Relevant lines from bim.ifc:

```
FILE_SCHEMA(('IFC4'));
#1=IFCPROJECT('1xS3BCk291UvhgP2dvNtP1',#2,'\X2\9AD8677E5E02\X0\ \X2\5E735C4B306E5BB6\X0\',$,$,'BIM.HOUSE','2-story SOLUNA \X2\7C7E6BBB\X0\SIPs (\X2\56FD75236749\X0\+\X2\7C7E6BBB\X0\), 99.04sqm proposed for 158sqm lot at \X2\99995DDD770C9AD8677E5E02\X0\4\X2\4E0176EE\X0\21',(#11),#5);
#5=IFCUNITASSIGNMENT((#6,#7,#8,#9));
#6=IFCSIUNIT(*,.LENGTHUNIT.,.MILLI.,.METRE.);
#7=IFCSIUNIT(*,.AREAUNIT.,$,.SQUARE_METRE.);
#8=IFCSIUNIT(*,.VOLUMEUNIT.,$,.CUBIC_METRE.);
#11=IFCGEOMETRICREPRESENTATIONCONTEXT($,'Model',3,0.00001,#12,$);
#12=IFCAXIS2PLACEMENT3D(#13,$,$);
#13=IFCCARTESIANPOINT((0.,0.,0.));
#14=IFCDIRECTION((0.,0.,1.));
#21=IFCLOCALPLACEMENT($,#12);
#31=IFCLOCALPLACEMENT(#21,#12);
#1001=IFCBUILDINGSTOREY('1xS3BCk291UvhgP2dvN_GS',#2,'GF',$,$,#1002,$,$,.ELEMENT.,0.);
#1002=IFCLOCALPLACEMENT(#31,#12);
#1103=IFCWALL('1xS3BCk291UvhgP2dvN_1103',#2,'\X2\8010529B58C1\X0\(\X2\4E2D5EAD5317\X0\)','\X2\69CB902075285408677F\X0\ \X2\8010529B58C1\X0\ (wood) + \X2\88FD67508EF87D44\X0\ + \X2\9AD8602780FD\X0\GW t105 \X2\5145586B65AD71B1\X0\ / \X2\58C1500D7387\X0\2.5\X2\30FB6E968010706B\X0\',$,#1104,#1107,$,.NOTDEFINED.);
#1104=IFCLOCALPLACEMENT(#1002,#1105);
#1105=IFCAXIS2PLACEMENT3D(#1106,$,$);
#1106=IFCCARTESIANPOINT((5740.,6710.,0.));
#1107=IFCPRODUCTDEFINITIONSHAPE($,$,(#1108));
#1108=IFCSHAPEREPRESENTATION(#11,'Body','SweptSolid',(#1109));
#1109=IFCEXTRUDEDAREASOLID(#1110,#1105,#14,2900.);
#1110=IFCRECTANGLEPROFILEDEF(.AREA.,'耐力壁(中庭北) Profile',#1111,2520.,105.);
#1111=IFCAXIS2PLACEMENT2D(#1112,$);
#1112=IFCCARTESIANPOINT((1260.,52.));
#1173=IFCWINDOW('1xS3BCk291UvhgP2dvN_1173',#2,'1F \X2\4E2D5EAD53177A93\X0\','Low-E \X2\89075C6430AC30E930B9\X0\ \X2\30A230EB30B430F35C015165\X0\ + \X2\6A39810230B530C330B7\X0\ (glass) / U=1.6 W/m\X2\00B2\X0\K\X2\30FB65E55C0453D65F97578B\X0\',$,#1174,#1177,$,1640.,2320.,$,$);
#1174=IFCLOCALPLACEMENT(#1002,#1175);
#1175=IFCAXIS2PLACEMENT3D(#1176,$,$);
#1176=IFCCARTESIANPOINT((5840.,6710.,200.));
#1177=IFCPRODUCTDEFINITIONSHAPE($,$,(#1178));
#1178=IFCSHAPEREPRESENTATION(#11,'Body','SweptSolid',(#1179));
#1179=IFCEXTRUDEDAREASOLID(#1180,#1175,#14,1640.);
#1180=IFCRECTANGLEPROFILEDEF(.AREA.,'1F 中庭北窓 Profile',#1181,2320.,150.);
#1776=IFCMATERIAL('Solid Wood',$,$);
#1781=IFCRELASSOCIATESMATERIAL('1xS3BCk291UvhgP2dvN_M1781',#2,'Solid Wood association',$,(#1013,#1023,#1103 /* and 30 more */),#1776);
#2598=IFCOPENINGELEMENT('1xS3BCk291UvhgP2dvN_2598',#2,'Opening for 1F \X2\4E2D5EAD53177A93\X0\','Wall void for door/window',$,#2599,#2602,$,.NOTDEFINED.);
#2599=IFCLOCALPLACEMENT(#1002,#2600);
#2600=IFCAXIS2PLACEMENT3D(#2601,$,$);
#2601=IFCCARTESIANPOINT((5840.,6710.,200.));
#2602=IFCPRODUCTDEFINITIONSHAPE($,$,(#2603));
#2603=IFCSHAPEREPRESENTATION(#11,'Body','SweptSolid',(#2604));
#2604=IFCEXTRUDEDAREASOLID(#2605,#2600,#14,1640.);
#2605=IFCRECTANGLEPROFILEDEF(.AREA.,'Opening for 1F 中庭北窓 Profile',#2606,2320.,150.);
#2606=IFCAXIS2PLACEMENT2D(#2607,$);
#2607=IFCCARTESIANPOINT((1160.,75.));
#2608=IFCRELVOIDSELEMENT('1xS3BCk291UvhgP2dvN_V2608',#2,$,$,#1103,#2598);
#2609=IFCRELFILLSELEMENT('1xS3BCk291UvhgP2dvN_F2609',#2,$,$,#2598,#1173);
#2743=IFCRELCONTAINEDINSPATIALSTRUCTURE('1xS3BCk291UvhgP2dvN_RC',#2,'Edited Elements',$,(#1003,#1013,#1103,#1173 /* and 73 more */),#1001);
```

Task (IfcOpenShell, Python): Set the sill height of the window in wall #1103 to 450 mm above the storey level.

```python
import numpy as np
import ifcopenshell
import ifcopenshell.api.geometry
import ifcopenshell.geom
import ifcopenshell.util.element
import ifcopenshell.util.placement
import ifcopenshell.util.shape
import ifcopenshell.util.unit

model = ifcopenshell.open("bim.ifc")
unit_scale = ifcopenshell.util.unit.calculate_unit_scale(model)

window = model.by_guid("1xS3BCk291UvhgP2dvN_1173")
opening = window.FillsVoids[0].RelatingOpeningElement
storey = ifcopenshell.util.element.get_container(window, ifc_class="IfcBuildingStorey")
level = ifcopenshell.util.placement.get_local_placement(storey.ObjectPlacement)[2, 3]

# The opening's origin need not be at the sill, so measure its lowest point.
shape = ifcopenshell.geom.create_shape(ifcopenshell.geom.settings(), opening)
bottom = ifcopenshell.util.shape.get_shape_bottom_elevation(shape, shape.geometry) / unit_scale
dz = level + 0.45 / unit_scale - bottom

shift = np.array([0.0, 0.0, dz])
# The window is not placed relative to its opening, so move both.
for product in (opening, window):
    matrix = ifcopenshell.util.placement.get_local_placement(product.ObjectPlacement)
    matrix[:3, 3] += shift
    ifcopenshell.api.geometry.edit_object_placement(model, product=product, matrix=matrix, is_si=False)

print(f"moved by {dz * unit_scale:+.3f} m")

model.write("bim_edited.ifc")
```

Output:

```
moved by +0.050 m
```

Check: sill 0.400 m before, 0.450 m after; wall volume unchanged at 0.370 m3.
